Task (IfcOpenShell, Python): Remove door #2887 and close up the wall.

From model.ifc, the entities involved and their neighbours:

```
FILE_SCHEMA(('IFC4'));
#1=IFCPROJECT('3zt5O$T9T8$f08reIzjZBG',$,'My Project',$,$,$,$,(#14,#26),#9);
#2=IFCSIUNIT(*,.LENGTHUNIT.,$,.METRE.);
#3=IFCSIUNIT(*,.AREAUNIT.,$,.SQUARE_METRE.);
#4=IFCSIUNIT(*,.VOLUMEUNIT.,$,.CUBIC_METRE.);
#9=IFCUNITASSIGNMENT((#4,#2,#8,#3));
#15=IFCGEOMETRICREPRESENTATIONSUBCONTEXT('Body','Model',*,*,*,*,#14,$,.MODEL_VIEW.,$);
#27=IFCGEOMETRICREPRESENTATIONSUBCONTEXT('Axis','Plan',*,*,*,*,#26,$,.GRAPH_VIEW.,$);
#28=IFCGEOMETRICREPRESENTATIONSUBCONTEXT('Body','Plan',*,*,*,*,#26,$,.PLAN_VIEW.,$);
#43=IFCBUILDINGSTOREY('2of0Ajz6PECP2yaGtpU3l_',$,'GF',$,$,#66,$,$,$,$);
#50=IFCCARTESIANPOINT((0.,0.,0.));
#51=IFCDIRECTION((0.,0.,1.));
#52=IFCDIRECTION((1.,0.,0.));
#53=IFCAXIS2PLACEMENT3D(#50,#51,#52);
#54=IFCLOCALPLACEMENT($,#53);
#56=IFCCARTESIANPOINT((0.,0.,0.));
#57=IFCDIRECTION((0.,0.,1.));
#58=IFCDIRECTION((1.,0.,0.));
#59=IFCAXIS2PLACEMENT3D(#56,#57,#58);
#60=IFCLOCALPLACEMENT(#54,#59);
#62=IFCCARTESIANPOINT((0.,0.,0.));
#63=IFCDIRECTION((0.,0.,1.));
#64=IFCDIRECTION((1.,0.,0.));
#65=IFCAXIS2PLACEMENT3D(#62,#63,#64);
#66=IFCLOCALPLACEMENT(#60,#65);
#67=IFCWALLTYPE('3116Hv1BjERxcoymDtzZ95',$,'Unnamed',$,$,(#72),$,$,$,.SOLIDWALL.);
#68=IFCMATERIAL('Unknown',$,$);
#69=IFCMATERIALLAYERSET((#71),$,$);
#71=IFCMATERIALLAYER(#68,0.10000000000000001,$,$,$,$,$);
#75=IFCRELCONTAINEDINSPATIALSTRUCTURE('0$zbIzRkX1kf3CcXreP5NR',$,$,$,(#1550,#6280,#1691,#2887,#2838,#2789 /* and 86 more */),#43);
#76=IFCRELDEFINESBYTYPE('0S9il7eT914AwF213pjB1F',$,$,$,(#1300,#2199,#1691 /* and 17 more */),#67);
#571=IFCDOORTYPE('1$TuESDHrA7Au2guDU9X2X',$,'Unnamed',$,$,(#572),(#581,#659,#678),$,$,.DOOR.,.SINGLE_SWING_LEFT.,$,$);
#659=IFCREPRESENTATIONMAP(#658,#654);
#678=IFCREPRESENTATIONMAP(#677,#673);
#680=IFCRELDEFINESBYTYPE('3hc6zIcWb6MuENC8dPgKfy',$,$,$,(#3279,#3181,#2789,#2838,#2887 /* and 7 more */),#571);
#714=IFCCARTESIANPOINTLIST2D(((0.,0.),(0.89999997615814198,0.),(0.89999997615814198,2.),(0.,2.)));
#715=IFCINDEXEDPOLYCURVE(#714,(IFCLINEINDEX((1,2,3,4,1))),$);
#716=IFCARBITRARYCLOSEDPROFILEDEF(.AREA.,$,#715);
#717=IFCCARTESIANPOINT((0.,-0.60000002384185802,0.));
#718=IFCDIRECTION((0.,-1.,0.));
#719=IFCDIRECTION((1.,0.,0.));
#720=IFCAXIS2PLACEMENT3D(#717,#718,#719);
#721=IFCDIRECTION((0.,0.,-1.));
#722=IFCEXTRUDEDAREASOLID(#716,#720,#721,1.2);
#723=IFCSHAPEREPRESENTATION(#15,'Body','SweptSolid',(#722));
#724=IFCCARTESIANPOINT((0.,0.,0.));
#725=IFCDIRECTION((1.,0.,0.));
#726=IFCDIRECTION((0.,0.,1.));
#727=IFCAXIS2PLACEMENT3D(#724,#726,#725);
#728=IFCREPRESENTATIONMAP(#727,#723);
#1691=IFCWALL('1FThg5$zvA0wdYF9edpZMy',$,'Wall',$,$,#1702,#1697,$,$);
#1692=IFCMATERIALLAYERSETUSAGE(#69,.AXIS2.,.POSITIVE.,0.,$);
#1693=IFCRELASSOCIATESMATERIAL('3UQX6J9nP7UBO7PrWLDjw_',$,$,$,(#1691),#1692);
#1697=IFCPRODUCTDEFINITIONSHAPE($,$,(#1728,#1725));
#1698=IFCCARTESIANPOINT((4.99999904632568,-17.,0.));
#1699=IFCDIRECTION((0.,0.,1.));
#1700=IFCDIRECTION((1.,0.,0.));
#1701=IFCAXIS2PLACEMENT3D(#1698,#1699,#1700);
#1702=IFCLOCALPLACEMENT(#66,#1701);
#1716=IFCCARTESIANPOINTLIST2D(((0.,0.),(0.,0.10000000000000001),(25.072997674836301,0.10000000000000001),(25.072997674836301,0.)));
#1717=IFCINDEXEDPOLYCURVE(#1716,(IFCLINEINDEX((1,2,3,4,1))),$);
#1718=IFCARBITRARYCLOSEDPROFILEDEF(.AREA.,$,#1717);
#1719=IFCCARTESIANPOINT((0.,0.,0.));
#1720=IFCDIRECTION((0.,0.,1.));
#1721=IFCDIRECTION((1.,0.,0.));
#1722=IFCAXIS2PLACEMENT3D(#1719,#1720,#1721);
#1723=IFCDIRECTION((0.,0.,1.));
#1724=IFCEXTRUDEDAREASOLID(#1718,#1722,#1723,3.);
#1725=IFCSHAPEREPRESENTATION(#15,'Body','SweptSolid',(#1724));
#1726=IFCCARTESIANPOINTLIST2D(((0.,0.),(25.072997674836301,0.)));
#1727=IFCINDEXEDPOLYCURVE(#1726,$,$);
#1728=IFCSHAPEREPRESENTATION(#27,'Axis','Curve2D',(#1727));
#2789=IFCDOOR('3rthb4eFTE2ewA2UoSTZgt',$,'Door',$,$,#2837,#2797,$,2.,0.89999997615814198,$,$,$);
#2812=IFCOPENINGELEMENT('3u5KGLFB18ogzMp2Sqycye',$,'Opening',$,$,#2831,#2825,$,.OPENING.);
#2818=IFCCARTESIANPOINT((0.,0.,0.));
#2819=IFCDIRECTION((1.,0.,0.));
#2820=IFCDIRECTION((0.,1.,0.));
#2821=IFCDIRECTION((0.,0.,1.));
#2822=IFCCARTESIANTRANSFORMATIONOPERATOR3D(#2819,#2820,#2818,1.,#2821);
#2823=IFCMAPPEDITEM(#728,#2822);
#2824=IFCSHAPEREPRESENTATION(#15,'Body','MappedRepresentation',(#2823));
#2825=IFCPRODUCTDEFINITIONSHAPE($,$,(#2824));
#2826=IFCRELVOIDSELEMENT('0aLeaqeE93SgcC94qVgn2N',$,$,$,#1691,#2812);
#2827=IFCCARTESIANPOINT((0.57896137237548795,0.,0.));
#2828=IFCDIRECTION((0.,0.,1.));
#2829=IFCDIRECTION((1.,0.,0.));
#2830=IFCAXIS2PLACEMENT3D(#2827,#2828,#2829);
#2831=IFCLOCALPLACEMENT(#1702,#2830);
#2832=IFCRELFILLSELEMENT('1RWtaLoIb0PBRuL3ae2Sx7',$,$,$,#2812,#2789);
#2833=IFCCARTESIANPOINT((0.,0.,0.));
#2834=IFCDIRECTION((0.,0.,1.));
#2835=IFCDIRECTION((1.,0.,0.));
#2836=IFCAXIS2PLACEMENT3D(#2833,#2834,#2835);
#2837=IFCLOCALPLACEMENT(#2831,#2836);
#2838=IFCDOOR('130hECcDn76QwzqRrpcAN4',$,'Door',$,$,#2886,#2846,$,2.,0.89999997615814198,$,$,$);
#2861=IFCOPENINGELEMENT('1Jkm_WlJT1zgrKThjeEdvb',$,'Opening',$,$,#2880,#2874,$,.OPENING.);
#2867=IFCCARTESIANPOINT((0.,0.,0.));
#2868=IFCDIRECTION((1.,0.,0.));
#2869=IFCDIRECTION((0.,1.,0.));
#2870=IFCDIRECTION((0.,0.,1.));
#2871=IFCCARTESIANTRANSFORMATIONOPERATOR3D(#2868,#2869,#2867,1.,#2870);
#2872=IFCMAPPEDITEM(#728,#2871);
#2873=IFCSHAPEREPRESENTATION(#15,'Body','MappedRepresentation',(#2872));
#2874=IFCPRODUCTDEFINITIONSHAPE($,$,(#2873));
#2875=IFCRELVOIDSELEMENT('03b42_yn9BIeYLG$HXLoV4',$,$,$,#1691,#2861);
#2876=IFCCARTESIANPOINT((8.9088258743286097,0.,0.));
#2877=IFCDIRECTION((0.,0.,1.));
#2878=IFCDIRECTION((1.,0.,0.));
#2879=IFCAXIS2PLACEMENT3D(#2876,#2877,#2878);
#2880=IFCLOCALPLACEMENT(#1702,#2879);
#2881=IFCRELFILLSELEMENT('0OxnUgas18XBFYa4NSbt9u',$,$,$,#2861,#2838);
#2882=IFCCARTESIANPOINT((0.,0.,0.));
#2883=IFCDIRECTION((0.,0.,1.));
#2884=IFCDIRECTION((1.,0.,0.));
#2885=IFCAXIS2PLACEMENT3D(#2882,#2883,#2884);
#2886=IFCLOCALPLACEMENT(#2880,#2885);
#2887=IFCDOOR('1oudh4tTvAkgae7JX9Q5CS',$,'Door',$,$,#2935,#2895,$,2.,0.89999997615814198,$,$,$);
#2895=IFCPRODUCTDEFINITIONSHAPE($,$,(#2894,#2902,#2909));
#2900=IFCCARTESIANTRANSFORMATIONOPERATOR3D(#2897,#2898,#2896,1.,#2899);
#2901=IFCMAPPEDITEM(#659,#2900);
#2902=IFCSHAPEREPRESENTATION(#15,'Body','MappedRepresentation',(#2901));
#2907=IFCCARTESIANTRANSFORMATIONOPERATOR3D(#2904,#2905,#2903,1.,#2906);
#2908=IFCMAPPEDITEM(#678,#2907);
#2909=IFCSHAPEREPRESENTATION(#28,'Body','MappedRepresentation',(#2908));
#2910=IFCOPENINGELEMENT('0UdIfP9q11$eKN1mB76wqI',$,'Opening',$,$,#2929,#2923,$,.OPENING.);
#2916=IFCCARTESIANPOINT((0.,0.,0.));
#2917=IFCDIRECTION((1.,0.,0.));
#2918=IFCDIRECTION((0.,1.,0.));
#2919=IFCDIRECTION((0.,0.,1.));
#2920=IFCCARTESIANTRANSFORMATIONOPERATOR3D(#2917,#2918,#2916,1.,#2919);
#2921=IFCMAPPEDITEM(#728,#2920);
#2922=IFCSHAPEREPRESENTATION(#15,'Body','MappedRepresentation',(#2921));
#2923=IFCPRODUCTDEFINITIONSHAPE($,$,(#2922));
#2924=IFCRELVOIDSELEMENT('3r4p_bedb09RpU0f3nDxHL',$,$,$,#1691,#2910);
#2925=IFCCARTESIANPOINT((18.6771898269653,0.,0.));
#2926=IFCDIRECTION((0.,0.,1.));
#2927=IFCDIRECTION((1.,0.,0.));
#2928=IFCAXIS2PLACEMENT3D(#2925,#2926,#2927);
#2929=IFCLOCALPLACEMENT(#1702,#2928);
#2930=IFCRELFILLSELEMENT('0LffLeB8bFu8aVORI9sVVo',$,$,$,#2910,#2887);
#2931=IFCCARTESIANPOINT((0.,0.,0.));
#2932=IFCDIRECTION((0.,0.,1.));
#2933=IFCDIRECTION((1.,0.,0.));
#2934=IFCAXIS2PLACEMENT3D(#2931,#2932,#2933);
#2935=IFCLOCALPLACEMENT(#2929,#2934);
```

```python
import ifcopenshell
import ifcopenshell.api.feature
import ifcopenshell.api.root
import ifcopenshell.geom
import ifcopenshell.util.shape

model = ifcopenshell.open("model.ifc")
settings = ifcopenshell.geom.settings()


def volume(element):
    """Net volume in cubic metres, openings subtracted."""
    shape = ifcopenshell.geom.create_shape(settings, element)
    return ifcopenshell.util.shape.get_volume(shape.geometry)


door = model.by_guid("1oudh4tTvAkgae7JX9Q5CS")
opening = door.FillsVoids[0].RelatingOpeningElement
wall = opening.VoidsElements[0].RelatingBuildingElement
before = volume(wall)

ifcopenshell.api.root.remove_product(model, product=door)
ifcopenshell.api.feature.remove_feature(model, feature=opening)

after = volume(wall)

print(f"wall volume {before:.3f} -> {after:.3f} m3")

model.write("model_rev.ifc")
```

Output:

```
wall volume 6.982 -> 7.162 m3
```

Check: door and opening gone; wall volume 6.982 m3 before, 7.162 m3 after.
